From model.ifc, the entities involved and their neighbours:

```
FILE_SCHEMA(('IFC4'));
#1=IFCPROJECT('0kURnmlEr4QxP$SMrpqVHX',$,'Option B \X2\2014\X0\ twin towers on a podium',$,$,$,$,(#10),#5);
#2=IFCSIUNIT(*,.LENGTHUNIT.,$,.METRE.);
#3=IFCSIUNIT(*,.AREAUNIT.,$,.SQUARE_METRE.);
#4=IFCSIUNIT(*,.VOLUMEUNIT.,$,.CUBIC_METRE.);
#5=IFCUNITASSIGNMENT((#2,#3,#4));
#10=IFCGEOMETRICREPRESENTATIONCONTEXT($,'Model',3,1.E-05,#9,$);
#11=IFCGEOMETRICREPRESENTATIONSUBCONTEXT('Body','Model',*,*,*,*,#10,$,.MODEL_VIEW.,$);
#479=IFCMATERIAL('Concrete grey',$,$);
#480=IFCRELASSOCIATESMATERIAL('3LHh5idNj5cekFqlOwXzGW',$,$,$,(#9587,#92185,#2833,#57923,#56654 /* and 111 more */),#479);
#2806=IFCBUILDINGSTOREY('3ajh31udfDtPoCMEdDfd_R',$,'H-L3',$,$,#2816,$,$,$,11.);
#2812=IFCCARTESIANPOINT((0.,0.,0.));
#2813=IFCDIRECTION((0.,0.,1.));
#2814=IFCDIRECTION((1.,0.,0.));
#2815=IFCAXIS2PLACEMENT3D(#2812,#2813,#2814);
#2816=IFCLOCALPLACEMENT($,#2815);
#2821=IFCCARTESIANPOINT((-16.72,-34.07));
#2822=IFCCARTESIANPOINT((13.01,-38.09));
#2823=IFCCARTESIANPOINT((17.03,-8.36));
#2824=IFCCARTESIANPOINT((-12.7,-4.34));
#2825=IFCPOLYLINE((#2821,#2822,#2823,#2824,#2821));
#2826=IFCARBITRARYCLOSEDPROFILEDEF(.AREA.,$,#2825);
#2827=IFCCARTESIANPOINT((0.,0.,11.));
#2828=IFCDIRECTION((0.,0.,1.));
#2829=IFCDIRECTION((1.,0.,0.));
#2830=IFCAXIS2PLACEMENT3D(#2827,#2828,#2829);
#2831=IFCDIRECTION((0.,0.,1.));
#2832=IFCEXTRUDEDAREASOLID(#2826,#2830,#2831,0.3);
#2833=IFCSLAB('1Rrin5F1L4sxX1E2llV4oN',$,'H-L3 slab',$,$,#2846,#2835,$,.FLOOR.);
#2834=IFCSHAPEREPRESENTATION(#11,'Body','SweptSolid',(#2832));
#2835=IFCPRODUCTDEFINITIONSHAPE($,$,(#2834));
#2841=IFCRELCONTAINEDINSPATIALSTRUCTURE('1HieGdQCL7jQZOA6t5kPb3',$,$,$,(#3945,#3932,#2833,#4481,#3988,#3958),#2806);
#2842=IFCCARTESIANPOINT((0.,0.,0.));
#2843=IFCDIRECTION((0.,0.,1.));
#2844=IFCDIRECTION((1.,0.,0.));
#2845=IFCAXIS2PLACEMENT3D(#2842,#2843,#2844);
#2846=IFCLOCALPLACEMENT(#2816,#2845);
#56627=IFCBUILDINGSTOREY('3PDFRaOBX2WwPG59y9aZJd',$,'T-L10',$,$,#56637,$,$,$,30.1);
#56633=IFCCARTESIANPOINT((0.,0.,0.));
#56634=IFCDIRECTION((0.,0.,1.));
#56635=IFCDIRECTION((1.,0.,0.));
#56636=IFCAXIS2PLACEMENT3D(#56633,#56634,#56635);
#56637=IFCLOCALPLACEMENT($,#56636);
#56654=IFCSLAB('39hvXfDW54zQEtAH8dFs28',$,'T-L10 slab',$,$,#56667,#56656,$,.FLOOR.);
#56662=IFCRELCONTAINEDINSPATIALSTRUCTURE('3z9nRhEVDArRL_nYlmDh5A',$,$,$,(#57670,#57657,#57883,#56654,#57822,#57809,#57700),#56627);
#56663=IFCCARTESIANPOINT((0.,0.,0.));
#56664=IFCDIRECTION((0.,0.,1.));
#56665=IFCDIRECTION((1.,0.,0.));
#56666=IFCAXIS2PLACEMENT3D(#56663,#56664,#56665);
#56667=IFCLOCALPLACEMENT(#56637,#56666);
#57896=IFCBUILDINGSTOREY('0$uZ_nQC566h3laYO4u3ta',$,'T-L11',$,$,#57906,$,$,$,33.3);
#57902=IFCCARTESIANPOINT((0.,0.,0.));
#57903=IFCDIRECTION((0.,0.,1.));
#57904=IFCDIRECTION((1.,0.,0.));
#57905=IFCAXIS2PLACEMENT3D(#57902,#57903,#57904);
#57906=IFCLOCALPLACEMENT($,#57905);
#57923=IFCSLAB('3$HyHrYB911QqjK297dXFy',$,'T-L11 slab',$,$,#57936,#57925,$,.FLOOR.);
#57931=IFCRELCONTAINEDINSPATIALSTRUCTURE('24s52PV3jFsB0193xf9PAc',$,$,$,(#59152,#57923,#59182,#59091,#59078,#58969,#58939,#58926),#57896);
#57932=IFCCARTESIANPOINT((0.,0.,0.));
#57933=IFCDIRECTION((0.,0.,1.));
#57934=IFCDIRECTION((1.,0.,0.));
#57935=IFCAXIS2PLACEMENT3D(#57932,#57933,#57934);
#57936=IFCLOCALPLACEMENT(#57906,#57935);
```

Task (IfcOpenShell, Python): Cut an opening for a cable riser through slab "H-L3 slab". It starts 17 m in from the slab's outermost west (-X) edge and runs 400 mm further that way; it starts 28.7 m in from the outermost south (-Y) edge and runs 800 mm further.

```python
import numpy as np
import ifcopenshell
import ifcopenshell.api.feature
import ifcopenshell.api.geometry
import ifcopenshell.api.root
import ifcopenshell.geom
import ifcopenshell.util.placement
import ifcopenshell.util.representation
import ifcopenshell.util.shape
import ifcopenshell.util.unit

model = ifcopenshell.open("model.ifc")
unit_scale = ifcopenshell.util.unit.calculate_unit_scale(model)
settings = ifcopenshell.geom.settings()


def volume(element):
    """Net volume in cubic metres, openings subtracted."""
    shape = ifcopenshell.geom.create_shape(settings, element)
    return ifcopenshell.util.shape.get_volume(shape.geometry)


slab = model.by_guid("1Rrin5F1L4sxX1E2llV4oN")
before = volume(slab)

# Extent in the slab's own axes, in metres. The edges named are its -X and -Y sides.
slab_shape = ifcopenshell.geom.create_shape(settings, slab)
vertices = ifcopenshell.util.shape.get_vertices(slab_shape.geometry)
x_min, y_min, bottom = vertices.min(axis=0)
top = vertices[:, 2].max()

opening = ifcopenshell.api.root.create_entity(model, ifc_class="IfcOpeningElement", name="Cable riser opening", predefined_type="OPENING")
context = ifcopenshell.util.representation.get_context(model, "Model", "Body", "MODEL_VIEW")
width, depth = 0.4, 0.8
outline = [(0.0, 0.0), (width, 0.0), (width, depth), (0.0, depth), (0.0, 0.0)]
# Overshoot both faces by 50 mm so the cut is clean.
shape = ifcopenshell.api.geometry.add_slab_representation(
    model, context=context, depth=top - bottom + 0.1, polyline=outline
)
ifcopenshell.api.geometry.assign_representation(model, product=opening, representation=shape)

matrix = ifcopenshell.util.placement.get_local_placement(slab.ObjectPlacement)
matrix[:, 3] = matrix @ np.append(np.array([x_min + 17, y_min + 28.7, bottom - 0.05]) / unit_scale, 1.0)
ifcopenshell.api.geometry.edit_object_placement(model, product=opening, matrix=matrix, is_si=False)
ifcopenshell.api.feature.add_feature(model, feature=opening, element=slab)

after = volume(slab)

print(f"slab volume {before:.3f} -> {after:.3f} m3")

model.write("model_v2.ifc")
```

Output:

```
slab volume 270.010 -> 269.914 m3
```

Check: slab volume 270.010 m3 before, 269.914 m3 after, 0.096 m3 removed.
